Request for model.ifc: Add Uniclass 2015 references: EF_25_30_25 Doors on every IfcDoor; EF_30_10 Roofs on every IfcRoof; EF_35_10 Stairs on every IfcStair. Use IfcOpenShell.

First a look at what the model holds.

```python
import ifcopenshell

model = ifcopenshell.open("model.ifc")
print(model.schema)
print("classifications:", [c.Name for c in model.by_type("IfcClassification")])
for ifc_class in ("IfcDoor", "IfcRoof", "IfcStair", "IfcWall", "IfcWindow"):
    print(ifc_class, len(model.by_type(ifc_class)))
```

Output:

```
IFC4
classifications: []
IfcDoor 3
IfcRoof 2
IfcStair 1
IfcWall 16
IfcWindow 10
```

```python
import ifcopenshell
import ifcopenshell.api.classification

model = ifcopenshell.open("model.ifc")

system = ifcopenshell.api.classification.add_classification(model, classification="Uniclass 2015")

codes = {
    "IfcDoor": ("EF_25_30_25", "Doors"),
    "IfcRoof": ("EF_30_10", "Roofs"),
    "IfcStair": ("EF_35_10", "Stairs"),
}
for ifc_class, (code, name) in codes.items():
    products = model.by_type(ifc_class)
    ifcopenshell.api.classification.add_reference(
        model, products=products, classification=system, identification=code, name=name
    )
    print(code, len(products))

model.write("model-out.ifc")
```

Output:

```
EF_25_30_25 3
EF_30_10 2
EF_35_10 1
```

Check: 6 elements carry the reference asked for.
